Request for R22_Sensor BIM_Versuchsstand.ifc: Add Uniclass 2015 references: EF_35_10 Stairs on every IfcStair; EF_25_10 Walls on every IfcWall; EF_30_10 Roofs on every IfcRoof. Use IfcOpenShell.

First a look at what the model holds.

```python
import ifcopenshell

model = ifcopenshell.open("R22_Sensor BIM_Versuchsstand.ifc")
print(model.schema)
print("classifications:", [c.Name for c in model.by_type("IfcClassification")])
for ifc_class in ("IfcDoor", "IfcRoof", "IfcStair", "IfcWall", "IfcWindow"):
    print(ifc_class, len(model.by_type(ifc_class)))
```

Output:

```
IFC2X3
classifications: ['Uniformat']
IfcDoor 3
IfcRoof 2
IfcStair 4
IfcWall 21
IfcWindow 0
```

```python
import ifcopenshell
import ifcopenshell.api.classification

model = ifcopenshell.open("R22_Sensor BIM_Versuchsstand.ifc")

# IFC2X3 requires Source and Edition and has no link from the project to the system.
system = model.create_entity("IfcClassification", Source="NBS", Edition="2015", Name="Uniclass 2015")

codes = {
    "IfcStair": ("EF_35_10", "Stairs"),
    "IfcWall": ("EF_25_10", "Walls"),
    "IfcRoof": ("EF_30_10", "Roofs"),
}
for ifc_class, (code, name) in codes.items():
    products = model.by_type(ifc_class)
    ifcopenshell.api.classification.add_reference(
        model, products=products, classification=system, identification=code, name=name
    )
    print(code, len(products))

model.write("R22_Sensor BIM_Versuchsstand_rev.ifc")
```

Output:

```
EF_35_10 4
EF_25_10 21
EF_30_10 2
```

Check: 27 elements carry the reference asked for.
